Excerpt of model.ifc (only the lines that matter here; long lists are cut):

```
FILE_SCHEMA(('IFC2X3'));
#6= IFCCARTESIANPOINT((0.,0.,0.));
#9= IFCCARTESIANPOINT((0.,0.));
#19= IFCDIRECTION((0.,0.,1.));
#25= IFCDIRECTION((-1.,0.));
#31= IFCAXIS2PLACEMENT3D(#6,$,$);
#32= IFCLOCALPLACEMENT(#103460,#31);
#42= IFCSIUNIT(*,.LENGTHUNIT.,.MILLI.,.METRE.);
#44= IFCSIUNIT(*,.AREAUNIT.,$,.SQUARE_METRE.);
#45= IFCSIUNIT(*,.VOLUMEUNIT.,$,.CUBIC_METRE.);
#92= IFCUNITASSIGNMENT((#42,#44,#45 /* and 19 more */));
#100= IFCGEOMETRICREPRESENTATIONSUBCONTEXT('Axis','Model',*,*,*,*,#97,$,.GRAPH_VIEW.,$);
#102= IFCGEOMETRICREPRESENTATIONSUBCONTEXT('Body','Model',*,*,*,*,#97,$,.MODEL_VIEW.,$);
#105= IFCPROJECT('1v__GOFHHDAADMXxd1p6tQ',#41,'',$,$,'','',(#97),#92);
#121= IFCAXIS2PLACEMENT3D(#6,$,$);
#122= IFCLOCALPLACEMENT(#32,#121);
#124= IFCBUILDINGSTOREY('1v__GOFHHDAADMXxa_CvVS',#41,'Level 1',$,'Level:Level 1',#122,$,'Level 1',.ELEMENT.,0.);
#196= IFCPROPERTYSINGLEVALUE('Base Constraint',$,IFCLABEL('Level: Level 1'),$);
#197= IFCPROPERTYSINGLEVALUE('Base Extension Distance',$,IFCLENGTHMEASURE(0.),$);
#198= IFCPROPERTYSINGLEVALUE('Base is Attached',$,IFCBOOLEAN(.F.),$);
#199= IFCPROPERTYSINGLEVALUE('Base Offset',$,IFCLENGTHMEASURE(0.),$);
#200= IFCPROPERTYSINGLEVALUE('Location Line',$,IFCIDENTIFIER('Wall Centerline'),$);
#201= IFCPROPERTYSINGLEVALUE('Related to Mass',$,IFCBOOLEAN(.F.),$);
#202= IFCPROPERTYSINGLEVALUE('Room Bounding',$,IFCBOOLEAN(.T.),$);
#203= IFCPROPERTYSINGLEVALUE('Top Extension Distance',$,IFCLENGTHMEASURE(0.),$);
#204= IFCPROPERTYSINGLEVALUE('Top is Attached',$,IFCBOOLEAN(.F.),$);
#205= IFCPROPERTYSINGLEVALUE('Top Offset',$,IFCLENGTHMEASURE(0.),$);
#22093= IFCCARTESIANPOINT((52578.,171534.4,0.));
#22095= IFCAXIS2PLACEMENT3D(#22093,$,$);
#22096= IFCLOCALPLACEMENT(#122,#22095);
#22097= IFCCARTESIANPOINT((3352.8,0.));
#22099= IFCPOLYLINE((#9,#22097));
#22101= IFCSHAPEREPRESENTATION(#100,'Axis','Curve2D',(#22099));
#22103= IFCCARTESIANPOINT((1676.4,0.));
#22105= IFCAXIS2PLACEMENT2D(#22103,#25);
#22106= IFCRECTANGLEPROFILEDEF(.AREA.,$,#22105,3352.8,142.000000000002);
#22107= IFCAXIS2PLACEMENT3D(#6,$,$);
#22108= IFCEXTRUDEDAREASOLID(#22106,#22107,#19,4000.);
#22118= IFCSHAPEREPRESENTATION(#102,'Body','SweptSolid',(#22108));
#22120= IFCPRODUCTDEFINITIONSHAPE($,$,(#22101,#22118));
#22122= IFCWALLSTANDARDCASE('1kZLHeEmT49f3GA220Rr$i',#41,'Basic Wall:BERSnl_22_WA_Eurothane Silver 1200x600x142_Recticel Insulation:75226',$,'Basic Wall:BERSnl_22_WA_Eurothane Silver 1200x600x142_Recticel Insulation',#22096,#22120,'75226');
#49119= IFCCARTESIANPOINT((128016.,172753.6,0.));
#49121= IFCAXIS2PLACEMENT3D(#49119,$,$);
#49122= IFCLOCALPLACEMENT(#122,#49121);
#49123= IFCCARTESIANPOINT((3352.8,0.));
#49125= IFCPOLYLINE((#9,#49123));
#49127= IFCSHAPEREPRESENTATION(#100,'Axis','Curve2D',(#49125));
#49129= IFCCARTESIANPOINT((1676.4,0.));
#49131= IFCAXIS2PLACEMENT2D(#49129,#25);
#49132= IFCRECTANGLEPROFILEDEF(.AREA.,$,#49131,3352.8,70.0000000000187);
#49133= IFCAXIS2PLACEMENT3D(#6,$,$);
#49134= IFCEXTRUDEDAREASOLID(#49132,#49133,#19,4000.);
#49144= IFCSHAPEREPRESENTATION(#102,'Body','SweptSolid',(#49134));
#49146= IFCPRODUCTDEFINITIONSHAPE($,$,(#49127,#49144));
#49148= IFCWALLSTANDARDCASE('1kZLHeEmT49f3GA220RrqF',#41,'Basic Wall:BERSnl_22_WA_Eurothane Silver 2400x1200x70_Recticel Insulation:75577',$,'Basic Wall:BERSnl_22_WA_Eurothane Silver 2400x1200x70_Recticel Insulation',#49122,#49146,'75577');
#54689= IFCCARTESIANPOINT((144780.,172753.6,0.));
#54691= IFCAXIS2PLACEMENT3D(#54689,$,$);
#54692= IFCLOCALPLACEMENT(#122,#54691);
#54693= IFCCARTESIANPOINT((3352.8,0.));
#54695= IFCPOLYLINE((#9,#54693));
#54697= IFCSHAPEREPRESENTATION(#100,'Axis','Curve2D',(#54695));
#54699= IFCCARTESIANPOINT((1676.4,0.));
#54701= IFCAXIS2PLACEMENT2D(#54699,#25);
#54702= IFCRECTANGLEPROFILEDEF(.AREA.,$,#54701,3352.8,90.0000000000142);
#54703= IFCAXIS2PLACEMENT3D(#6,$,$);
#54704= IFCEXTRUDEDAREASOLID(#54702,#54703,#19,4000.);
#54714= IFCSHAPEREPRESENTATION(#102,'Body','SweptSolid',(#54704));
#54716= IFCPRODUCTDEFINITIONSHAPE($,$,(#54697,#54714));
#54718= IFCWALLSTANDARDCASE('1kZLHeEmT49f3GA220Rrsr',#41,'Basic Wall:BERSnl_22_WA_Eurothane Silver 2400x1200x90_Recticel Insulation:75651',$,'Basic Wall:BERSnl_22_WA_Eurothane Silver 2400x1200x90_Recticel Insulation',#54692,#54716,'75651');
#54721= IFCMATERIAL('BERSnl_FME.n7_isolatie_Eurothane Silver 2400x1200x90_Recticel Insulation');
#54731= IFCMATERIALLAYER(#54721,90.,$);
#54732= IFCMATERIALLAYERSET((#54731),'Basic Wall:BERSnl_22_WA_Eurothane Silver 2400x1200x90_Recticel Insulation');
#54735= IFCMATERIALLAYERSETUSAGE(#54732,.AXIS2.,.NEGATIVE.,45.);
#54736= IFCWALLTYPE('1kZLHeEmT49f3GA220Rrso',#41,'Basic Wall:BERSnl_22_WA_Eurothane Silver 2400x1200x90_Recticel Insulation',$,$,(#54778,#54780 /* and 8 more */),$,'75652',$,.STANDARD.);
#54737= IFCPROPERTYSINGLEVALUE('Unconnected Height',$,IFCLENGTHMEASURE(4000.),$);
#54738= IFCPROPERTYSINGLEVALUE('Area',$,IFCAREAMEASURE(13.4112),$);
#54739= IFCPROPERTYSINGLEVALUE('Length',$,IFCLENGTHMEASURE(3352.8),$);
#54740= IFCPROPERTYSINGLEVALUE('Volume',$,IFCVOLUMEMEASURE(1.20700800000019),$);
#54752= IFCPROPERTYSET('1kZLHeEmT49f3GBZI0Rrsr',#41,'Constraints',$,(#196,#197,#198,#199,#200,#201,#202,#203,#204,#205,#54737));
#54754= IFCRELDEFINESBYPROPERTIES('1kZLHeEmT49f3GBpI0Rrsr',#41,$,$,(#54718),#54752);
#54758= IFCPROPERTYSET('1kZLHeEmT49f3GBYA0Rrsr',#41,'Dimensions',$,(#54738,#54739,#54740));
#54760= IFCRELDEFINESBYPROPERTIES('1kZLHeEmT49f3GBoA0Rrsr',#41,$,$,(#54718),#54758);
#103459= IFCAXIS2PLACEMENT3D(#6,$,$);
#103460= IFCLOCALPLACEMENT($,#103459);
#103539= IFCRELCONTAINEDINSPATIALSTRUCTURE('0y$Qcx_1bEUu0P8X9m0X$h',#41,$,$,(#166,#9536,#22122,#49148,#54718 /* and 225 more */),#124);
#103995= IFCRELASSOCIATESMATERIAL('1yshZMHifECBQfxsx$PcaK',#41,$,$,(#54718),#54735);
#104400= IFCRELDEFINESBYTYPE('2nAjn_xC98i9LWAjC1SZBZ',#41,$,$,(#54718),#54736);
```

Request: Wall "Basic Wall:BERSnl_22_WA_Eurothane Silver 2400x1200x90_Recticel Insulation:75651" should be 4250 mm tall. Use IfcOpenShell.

```python
import ifcopenshell
import ifcopenshell.api.pset
import ifcopenshell.geom
import ifcopenshell.util.element
import ifcopenshell.util.representation
import ifcopenshell.util.shape
import ifcopenshell.util.unit

model = ifcopenshell.open("model.ifc")
unit_scale = ifcopenshell.util.unit.calculate_unit_scale(model)
area_scale = ifcopenshell.util.unit.calculate_unit_scale(model, "AREAUNIT")
volume_scale = ifcopenshell.util.unit.calculate_unit_scale(model, "VOLUMEUNIT")
settings = ifcopenshell.geom.settings()


def volume(element):
    """Net volume in cubic metres, openings subtracted."""
    shape = ifcopenshell.geom.create_shape(settings, element)
    return ifcopenshell.util.shape.get_volume(shape.geometry)


wall = model.by_guid("1kZLHeEmT49f3GA220Rrsr")
before = volume(wall)

body = ifcopenshell.util.representation.get_representation(wall, "Model", "Body")
solid = body.Items[0]
old_height = solid.Depth
solid.Depth = 4.25 / unit_scale
after = volume(wall)
thickness = 0.09  # wall thickness in metres

# Update the stored height, areas and volumes.
pset = model.by_id(ifcopenshell.util.element.get_pset(wall, "Constraints", should_inherit=False)["id"])
ifcopenshell.api.pset.edit_pset(model, pset=pset, properties={
    "Unconnected Height": model.create_entity("IfcLengthMeasure", solid.Depth),
})
pset = model.by_id(ifcopenshell.util.element.get_pset(wall, "Dimensions", should_inherit=False)["id"])
ifcopenshell.api.pset.edit_pset(model, pset=pset, properties={
    "Area": model.create_entity("IfcAreaMeasure", after / thickness / area_scale),
    "Volume": model.create_entity("IfcVolumeMeasure", after / volume_scale),
})

print(f"height {old_height:g} -> {solid.Depth:g}, volume {before:.3f} -> {after:.3f} m3")

model.write("model_updated.ifc")
```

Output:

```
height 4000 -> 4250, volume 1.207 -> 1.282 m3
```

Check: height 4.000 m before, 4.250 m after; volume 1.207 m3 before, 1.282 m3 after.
